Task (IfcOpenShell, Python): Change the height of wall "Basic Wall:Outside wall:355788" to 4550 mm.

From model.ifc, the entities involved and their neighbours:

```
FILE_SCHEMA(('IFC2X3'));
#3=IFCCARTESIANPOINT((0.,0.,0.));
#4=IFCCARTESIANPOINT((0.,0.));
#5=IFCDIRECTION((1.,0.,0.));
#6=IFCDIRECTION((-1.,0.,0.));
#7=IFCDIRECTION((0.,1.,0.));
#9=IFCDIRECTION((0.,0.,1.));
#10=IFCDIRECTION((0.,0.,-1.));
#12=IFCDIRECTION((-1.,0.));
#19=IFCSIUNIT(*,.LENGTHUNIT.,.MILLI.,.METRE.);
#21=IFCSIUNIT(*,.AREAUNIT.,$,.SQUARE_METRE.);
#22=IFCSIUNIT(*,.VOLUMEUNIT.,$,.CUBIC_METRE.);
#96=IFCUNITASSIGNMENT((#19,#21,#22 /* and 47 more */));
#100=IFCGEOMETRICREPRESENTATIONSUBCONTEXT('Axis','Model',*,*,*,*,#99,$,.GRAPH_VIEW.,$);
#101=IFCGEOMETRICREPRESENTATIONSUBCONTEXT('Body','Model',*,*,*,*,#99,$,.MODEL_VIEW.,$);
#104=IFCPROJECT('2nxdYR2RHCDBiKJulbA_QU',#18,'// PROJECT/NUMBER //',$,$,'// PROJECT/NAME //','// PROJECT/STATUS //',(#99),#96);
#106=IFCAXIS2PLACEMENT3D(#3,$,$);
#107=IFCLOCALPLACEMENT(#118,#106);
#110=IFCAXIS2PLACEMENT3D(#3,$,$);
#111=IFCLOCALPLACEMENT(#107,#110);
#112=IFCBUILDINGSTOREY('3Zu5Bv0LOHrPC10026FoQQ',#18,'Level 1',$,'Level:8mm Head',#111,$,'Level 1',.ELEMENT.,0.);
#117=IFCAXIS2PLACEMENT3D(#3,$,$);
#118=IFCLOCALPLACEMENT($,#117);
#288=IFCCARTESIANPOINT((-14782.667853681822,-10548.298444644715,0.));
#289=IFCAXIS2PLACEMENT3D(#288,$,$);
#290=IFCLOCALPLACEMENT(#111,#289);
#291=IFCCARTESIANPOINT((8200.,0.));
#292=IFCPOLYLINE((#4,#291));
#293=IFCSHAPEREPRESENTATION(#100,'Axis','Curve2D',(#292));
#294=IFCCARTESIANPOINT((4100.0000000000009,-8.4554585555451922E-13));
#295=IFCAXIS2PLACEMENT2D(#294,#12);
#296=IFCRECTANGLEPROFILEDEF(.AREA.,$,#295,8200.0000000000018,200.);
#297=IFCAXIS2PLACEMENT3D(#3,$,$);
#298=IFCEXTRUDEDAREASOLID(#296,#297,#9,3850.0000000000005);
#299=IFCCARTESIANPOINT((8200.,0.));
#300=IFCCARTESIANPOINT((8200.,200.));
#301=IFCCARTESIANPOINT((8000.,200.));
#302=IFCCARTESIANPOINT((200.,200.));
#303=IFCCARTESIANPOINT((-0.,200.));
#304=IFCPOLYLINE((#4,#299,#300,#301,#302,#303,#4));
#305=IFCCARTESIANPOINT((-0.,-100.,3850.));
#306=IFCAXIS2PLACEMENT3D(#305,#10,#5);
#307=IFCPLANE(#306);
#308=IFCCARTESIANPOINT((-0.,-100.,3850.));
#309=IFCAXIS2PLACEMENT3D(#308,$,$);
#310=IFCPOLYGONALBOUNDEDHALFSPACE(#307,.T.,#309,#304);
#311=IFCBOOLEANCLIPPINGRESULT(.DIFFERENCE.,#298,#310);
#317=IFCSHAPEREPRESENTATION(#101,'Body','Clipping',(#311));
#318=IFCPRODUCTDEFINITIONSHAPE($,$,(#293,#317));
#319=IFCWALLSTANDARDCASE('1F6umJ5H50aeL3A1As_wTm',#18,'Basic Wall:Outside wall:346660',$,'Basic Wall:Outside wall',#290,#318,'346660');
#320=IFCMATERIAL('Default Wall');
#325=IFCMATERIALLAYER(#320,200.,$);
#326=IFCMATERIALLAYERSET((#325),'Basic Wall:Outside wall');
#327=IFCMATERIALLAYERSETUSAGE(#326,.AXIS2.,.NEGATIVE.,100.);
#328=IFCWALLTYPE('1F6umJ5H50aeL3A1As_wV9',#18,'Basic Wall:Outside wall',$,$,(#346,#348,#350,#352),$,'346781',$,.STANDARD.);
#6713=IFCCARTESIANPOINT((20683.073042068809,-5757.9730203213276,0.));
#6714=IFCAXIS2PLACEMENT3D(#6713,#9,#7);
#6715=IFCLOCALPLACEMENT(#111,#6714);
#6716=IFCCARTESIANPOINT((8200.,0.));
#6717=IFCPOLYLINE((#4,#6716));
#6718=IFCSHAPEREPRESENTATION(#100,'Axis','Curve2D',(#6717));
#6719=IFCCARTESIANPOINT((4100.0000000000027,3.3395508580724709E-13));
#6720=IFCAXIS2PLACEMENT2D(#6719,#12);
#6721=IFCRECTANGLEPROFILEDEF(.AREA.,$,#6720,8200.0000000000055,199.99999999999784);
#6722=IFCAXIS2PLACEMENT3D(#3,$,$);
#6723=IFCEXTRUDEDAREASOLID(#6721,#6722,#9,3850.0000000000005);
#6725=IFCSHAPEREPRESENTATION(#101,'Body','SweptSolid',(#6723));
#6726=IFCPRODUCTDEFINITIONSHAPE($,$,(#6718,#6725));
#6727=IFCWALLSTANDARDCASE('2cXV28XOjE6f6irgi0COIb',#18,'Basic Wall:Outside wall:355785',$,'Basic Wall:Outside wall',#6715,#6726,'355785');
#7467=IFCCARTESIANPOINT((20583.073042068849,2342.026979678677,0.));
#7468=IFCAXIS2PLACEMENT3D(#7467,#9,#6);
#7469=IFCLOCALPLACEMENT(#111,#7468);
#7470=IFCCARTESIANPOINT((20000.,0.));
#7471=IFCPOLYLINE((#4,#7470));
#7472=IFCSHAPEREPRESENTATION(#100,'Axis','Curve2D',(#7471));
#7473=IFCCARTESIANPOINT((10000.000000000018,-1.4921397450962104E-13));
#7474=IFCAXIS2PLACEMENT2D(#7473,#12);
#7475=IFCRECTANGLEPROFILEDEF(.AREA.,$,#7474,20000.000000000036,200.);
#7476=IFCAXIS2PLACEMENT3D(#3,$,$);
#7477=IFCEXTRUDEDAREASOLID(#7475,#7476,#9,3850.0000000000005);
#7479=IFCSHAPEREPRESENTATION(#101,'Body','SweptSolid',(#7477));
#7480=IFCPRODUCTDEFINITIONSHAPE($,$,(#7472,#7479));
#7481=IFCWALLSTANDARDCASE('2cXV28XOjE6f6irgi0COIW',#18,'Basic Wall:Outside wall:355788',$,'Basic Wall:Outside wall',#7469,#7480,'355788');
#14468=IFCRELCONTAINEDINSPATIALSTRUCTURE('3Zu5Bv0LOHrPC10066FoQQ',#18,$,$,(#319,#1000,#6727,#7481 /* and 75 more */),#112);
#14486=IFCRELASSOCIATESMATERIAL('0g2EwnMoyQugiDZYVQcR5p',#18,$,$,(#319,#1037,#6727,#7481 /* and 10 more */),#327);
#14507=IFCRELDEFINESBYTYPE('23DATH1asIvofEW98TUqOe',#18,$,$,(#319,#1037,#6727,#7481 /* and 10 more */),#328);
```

```python
import ifcopenshell
import ifcopenshell.geom
import ifcopenshell.util.representation
import ifcopenshell.util.shape
import ifcopenshell.util.unit

model = ifcopenshell.open("model.ifc")
unit_scale = ifcopenshell.util.unit.calculate_unit_scale(model)
settings = ifcopenshell.geom.settings()


def volume(element):
    """Net volume in cubic metres, openings subtracted."""
    shape = ifcopenshell.geom.create_shape(settings, element)
    return ifcopenshell.util.shape.get_volume(shape.geometry)


wall = model.by_guid("2cXV28XOjE6f6irgi0COIW")
before = volume(wall)

body = ifcopenshell.util.representation.get_representation(wall, "Model", "Body")
solid = body.Items[0]
old_height = solid.Depth
solid.Depth = 4.55 / unit_scale
after = volume(wall)

print(f"height {old_height:g} -> {solid.Depth:g}, volume {before:.3f} -> {after:.3f} m3")

model.write("model_rev.ifc")
```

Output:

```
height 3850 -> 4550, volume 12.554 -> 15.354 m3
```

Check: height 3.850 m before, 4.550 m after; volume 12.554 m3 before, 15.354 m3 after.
